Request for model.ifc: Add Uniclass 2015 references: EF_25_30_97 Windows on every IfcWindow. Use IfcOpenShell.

First a look at what the model holds.

```python
import ifcopenshell

model = ifcopenshell.open("model.ifc")
print(model.schema)
print("classifications:", [c.Name for c in model.by_type("IfcClassification")])
for ifc_class in ("IfcDoor", "IfcRoof", "IfcStair", "IfcWall", "IfcWindow"):
    print(ifc_class, len(model.by_type(ifc_class)))
```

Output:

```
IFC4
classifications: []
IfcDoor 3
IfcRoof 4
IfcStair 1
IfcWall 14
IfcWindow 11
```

```python
import ifcopenshell
import ifcopenshell.api.classification

model = ifcopenshell.open("model.ifc")

system = ifcopenshell.api.classification.add_classification(model, classification="Uniclass 2015")

codes = {
    "IfcWindow": ("EF_25_30_97", "Windows"),
}
for ifc_class, (code, name) in codes.items():
    products = model.by_type(ifc_class)
    ifcopenshell.api.classification.add_reference(
        model, products=products, classification=system, identification=code, name=name
    )
    print(code, len(products))

model.write("model-out.ifc")
```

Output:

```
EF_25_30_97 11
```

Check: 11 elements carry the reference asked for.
